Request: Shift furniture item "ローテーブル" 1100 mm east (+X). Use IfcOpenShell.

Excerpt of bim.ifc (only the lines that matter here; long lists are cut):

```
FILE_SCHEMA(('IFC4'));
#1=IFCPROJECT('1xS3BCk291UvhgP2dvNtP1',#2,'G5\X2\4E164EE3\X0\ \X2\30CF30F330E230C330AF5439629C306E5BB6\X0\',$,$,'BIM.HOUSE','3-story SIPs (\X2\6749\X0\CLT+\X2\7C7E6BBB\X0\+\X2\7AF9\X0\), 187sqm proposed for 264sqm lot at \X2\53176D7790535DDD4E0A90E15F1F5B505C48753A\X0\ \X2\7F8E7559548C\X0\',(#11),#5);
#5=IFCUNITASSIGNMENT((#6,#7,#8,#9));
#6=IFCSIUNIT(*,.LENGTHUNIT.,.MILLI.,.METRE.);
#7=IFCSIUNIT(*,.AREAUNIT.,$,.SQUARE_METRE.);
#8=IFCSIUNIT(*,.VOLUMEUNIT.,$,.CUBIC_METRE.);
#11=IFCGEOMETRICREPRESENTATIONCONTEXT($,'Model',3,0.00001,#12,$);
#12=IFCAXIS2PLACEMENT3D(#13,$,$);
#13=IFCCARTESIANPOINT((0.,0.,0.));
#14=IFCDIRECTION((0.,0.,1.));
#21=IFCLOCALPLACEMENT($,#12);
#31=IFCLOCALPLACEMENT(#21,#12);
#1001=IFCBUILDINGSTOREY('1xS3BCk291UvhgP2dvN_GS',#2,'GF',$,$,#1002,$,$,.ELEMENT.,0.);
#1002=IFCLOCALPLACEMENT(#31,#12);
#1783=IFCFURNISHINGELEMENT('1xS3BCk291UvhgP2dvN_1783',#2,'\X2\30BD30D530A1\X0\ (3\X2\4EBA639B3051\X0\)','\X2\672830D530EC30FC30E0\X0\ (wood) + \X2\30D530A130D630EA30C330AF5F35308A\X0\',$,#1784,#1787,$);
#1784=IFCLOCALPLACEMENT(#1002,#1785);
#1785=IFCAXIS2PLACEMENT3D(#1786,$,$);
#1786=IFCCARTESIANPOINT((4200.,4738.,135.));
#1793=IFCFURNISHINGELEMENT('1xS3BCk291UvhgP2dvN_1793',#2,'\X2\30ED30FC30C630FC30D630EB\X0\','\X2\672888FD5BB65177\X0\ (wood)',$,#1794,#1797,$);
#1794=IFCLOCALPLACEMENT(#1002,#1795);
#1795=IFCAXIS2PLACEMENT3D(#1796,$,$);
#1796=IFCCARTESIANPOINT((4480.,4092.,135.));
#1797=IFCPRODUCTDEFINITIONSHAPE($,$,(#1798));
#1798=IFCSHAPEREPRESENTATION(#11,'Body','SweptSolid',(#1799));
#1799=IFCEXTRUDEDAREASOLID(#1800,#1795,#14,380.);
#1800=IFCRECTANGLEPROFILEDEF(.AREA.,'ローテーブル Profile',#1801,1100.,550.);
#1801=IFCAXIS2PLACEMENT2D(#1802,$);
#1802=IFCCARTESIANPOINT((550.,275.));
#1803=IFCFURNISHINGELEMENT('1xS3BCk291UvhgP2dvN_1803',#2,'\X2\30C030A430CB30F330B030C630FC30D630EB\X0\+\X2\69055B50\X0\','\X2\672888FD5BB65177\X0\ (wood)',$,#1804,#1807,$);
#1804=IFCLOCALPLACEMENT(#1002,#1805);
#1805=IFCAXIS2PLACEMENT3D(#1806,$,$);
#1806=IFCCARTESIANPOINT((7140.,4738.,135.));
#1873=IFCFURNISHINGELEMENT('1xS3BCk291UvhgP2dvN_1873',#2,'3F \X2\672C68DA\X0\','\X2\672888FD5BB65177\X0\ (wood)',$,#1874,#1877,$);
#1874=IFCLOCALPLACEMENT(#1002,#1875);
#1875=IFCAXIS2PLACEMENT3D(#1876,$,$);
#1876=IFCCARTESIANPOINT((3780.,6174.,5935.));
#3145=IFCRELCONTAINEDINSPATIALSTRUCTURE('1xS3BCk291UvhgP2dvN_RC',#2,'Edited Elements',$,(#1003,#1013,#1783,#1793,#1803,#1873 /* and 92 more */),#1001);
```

```python
import ifcopenshell
import ifcopenshell.api.geometry
import ifcopenshell.util.placement
import ifcopenshell.util.unit

model = ifcopenshell.open("bim.ifc")
unit_scale = ifcopenshell.util.unit.calculate_unit_scale(model)

item = model.by_guid("1xS3BCk291UvhgP2dvN_1793")
matrix = ifcopenshell.util.placement.get_local_placement(item.ObjectPlacement)
matrix[0, 3] += 1.1 / unit_scale
ifcopenshell.api.geometry.edit_object_placement(model, product=item, matrix=matrix, is_si=False)

print(ifcopenshell.util.placement.get_local_placement(item.ObjectPlacement).round(3) + 0.0)

model.write("bim_v2.ifc")
```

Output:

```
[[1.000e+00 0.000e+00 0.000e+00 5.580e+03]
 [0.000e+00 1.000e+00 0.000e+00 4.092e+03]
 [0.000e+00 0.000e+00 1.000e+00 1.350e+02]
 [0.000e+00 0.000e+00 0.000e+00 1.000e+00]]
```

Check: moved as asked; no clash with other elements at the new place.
